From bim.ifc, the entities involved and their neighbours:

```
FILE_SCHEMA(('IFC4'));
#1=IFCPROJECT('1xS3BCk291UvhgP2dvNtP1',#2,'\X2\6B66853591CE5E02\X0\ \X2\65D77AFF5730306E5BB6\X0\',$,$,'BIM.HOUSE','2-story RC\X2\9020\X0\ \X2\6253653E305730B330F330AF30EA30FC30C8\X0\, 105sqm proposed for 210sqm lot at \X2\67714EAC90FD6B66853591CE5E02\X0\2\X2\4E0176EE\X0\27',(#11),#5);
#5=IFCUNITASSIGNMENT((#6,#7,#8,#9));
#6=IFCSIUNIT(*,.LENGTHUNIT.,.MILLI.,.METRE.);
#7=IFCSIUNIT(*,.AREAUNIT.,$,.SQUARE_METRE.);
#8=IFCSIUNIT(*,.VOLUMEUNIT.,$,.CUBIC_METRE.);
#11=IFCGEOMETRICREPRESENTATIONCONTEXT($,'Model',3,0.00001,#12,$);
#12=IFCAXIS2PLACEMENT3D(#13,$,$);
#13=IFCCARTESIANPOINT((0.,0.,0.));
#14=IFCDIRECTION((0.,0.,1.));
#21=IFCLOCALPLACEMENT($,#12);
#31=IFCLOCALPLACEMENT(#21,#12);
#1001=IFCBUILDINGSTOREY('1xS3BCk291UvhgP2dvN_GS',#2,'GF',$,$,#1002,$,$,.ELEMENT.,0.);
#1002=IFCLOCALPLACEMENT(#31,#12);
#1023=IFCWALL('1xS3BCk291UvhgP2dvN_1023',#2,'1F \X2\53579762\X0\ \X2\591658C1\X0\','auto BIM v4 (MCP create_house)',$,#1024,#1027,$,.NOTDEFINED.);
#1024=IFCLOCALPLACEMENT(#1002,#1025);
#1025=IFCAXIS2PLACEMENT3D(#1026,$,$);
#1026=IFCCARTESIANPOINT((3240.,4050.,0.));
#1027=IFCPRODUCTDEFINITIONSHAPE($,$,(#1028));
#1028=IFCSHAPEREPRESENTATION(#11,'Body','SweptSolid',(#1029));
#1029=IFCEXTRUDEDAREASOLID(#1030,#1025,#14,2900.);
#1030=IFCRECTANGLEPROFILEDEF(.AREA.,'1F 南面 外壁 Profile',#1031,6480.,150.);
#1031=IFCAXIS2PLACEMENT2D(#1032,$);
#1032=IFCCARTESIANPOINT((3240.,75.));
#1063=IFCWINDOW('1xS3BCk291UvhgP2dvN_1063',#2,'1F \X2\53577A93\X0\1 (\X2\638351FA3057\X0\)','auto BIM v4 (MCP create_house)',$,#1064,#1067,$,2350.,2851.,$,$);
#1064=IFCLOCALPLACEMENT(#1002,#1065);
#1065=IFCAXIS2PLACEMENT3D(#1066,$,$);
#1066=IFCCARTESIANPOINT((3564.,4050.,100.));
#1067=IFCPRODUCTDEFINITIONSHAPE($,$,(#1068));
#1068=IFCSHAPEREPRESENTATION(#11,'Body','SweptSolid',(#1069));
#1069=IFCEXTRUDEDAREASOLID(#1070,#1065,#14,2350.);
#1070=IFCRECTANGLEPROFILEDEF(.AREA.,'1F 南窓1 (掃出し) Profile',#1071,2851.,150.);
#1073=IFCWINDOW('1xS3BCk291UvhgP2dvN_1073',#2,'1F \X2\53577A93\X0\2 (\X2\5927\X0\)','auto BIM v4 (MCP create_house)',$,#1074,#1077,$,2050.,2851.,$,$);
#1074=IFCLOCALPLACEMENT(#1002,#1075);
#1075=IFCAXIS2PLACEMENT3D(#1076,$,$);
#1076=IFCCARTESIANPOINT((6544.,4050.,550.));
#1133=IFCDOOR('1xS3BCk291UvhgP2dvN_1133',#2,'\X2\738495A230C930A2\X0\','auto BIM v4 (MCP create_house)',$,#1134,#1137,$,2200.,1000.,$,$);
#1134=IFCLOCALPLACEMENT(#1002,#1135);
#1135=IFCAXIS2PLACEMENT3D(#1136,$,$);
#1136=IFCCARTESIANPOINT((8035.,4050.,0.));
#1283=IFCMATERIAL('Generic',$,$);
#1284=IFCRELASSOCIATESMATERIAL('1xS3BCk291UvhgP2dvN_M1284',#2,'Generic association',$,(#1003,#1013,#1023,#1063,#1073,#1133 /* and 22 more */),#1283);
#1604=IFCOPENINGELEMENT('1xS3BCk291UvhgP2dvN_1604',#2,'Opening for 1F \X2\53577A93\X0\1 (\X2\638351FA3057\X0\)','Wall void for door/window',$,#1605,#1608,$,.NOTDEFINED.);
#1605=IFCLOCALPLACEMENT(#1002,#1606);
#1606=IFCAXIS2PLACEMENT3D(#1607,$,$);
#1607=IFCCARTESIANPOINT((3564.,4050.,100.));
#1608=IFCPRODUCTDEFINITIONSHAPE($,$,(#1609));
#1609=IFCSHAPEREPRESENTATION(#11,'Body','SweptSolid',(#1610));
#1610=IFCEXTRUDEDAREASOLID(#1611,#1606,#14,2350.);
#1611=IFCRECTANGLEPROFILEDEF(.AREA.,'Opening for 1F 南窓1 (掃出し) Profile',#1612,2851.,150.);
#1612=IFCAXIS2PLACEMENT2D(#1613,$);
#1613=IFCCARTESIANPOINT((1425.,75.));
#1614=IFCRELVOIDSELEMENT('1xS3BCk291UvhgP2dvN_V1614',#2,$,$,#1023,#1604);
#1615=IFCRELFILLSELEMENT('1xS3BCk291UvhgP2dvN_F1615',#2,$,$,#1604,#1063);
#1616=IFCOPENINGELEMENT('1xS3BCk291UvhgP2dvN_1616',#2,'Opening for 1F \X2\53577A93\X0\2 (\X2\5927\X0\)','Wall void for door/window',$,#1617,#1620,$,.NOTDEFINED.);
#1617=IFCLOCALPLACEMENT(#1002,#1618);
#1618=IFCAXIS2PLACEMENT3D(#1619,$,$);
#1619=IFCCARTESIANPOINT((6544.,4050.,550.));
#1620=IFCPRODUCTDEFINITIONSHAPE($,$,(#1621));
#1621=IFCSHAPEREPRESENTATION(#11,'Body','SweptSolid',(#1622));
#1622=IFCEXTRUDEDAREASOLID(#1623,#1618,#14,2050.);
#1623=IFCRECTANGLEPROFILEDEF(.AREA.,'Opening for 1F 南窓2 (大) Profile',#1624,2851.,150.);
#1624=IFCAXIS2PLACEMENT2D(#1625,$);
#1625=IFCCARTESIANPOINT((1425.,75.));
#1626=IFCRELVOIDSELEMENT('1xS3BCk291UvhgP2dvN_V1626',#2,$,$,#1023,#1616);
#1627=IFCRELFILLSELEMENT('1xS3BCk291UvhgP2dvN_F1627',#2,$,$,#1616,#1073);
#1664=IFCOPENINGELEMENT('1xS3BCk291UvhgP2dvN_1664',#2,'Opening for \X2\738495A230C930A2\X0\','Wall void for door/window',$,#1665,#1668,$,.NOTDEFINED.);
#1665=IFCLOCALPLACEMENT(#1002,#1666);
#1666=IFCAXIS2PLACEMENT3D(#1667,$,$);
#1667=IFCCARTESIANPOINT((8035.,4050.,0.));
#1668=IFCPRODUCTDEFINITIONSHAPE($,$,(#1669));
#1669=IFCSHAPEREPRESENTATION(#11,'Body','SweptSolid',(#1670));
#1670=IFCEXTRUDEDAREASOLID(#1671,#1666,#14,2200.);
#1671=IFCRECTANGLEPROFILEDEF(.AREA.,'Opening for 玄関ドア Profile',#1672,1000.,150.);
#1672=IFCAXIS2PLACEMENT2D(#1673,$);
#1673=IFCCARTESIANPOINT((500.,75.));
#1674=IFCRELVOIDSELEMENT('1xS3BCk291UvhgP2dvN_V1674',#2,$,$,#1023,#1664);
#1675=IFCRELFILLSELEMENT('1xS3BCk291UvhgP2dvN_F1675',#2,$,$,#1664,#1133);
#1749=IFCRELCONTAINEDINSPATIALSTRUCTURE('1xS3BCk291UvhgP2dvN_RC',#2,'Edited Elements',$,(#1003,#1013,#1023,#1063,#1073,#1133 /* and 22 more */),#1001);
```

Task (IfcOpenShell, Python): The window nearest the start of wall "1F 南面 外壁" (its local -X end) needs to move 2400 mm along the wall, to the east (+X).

```python
import ifcopenshell
import ifcopenshell.api.geometry
import ifcopenshell.util.placement

model = ifcopenshell.open("bim.ifc")

window = model.by_id(1063)
opening = window.FillsVoids[0].RelatingOpeningElement
wall = opening.VoidsElements[0].RelatingBuildingElement

wall_matrix = ifcopenshell.util.placement.get_local_placement(wall.ObjectPlacement)
shift = wall_matrix[:3, 0] * 2400.0
before = ifcopenshell.util.placement.get_local_placement(window.ObjectPlacement)[:3, 3].copy()

# The window is not placed relative to its opening, so move both.
for product in (opening, window):
    matrix = ifcopenshell.util.placement.get_local_placement(product.ObjectPlacement)
    matrix[:3, 3] += shift
    ifcopenshell.api.geometry.edit_object_placement(model, product=product, matrix=matrix, is_si=False)

after = ifcopenshell.util.placement.get_local_placement(window.ObjectPlacement)[:3, 3]
print("window moved by", (after - before).round(3) + 0.0)

model.write("bim-out.ifc")
```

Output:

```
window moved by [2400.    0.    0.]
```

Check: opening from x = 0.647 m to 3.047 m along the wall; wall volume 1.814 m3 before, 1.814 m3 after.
